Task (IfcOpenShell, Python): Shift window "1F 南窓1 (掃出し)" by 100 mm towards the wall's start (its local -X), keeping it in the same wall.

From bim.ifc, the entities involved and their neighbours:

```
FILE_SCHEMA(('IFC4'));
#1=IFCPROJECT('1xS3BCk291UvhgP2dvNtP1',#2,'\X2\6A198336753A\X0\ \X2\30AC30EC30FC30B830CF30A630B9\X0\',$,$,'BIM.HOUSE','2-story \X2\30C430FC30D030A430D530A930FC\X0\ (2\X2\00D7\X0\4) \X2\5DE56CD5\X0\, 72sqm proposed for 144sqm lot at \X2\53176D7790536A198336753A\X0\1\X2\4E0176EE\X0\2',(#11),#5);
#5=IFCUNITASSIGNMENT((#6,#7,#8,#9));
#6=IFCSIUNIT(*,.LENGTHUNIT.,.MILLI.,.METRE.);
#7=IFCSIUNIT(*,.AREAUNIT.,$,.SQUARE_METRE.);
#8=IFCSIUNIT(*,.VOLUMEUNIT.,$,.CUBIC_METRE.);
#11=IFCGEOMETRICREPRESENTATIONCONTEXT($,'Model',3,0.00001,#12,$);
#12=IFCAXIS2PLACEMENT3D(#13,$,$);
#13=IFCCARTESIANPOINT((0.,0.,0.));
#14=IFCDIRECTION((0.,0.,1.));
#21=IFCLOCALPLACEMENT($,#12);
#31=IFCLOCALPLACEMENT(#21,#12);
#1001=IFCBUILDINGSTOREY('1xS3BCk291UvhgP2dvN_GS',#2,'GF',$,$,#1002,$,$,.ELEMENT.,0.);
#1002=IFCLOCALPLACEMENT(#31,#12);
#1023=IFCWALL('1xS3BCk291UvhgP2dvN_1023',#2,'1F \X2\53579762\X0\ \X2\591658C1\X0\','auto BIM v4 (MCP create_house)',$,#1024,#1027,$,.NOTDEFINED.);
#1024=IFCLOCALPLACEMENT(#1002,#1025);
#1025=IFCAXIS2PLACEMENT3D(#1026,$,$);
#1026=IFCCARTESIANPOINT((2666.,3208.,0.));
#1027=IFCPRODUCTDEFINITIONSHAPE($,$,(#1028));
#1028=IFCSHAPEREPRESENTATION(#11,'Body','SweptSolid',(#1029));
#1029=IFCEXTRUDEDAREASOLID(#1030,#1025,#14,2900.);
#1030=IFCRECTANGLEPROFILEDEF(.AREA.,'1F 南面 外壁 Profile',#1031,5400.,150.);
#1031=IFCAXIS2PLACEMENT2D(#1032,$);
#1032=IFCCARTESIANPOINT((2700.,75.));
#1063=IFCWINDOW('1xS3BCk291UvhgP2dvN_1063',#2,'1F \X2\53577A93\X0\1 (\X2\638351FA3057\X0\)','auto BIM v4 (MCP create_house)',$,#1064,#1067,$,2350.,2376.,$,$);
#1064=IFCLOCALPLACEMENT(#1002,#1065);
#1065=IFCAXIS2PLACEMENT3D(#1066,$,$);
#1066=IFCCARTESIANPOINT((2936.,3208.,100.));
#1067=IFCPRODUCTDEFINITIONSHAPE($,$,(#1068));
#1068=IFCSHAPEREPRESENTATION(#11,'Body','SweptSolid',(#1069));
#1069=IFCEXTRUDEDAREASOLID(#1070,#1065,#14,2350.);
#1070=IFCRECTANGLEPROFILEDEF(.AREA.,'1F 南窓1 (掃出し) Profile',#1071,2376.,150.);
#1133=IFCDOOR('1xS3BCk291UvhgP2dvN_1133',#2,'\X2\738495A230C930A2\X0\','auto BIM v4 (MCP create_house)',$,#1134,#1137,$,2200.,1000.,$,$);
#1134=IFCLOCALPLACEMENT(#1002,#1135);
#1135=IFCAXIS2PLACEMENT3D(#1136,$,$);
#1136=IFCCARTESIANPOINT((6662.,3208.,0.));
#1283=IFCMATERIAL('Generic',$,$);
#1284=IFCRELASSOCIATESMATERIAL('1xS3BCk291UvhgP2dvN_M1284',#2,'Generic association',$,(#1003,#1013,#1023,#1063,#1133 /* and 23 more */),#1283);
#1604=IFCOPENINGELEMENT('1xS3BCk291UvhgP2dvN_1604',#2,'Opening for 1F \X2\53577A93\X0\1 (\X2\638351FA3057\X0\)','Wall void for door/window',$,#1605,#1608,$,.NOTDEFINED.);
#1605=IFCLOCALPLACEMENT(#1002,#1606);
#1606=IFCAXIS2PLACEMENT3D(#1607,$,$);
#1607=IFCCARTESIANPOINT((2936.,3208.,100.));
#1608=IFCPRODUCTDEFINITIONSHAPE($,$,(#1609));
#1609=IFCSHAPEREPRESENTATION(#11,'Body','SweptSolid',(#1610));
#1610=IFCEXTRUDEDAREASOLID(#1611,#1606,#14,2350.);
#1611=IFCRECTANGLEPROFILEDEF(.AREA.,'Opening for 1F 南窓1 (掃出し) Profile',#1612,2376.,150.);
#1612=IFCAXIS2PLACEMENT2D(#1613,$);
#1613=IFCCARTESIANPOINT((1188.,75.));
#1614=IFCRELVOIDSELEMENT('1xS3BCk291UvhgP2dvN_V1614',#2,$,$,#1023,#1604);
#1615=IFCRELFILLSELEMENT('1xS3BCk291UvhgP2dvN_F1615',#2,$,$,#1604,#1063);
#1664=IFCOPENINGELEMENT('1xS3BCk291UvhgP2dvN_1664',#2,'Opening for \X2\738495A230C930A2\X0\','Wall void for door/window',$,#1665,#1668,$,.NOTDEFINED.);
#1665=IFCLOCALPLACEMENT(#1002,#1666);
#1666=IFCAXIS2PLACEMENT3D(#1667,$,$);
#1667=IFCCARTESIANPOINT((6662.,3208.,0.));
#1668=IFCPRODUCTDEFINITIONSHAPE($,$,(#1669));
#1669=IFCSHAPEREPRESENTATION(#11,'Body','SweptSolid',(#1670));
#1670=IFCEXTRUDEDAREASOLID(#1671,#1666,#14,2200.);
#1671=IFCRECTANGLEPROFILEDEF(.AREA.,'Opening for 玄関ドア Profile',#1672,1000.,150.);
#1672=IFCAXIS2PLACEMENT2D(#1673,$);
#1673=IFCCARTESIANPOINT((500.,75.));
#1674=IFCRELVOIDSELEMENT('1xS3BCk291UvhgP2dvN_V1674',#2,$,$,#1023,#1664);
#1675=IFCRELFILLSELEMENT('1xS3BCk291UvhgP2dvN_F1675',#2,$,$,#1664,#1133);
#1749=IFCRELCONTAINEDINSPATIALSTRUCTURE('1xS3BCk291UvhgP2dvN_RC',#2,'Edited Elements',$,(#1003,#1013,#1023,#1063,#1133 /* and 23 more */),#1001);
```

```python
import ifcopenshell
import ifcopenshell.api.geometry
import ifcopenshell.util.placement
import ifcopenshell.util.unit

model = ifcopenshell.open("bim.ifc")
unit_scale = ifcopenshell.util.unit.calculate_unit_scale(model)

window = model.by_guid("1xS3BCk291UvhgP2dvN_1063")
opening = window.FillsVoids[0].RelatingOpeningElement
wall = opening.VoidsElements[0].RelatingBuildingElement

wall_matrix = ifcopenshell.util.placement.get_local_placement(wall.ObjectPlacement)
shift = wall_matrix[:3, 0] * -0.1 / unit_scale
before = ifcopenshell.util.placement.get_local_placement(window.ObjectPlacement)[:3, 3].copy()

# The window is not placed relative to its opening, so move both.
for product in (opening, window):
    matrix = ifcopenshell.util.placement.get_local_placement(product.ObjectPlacement)
    matrix[:3, 3] += shift
    ifcopenshell.api.geometry.edit_object_placement(model, product=product, matrix=matrix, is_si=False)

after = ifcopenshell.util.placement.get_local_placement(window.ObjectPlacement)[:3, 3]
print("window moved by", (after - before).round(3) + 0.0)

model.write("bim_v2.ifc")
```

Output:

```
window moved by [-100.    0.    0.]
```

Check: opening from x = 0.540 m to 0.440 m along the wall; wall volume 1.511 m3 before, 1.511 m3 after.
